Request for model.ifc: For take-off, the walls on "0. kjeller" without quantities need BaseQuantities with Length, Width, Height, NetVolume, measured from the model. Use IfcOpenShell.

First a look at what the model holds.

```python
import ifcopenshell
import ifcopenshell.util.element
import ifcopenshell.util.unit

model = ifcopenshell.open("model.ifc")
print(model.schema)
for unit_type in ("LENGTHUNIT", "AREAUNIT", "VOLUMEUNIT"):
    print(unit_type, ifcopenshell.util.unit.calculate_unit_scale(model, unit_type))
storey = next(s for s in model.by_type("IfcBuildingStorey") if s.Name == "0. kjeller")
walls = [e for e in ifcopenshell.util.element.get_decomposition(storey) if e.is_a("IfcWall")]
for e in sorted(walls, key=lambda e: e.id()):
    print(e.id(), e.is_a(), e.Name, list(ifcopenshell.util.element.get_psets(e, qtos_only=True)), sep=" | ")
```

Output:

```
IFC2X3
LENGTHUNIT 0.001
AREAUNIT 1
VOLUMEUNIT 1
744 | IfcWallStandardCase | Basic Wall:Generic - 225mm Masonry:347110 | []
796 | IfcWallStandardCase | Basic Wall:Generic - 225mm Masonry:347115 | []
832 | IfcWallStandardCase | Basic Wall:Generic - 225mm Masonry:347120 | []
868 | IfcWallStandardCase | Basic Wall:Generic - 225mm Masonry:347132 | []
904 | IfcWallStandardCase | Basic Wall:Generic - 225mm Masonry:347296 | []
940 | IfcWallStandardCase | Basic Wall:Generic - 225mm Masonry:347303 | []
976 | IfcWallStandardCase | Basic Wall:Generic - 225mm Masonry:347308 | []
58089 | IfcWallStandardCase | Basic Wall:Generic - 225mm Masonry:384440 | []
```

```python
import ifcopenshell
import ifcopenshell.api.pset
import ifcopenshell.geom
import ifcopenshell.util.element
import ifcopenshell.util.shape
import ifcopenshell.util.unit

model = ifcopenshell.open("model.ifc")
unit_scale = ifcopenshell.util.unit.calculate_unit_scale(model)
volume_scale = ifcopenshell.util.unit.calculate_unit_scale(model, "VOLUMEUNIT")
settings = ifcopenshell.geom.settings()

storey = next(s for s in model.by_type("IfcBuildingStorey") if s.Name == "0. kjeller")
walls = [e for e in ifcopenshell.util.element.get_decomposition(storey) if e.is_a("IfcWall")]

for e in sorted(walls, key=lambda e: e.id()):
    if ifcopenshell.util.element.get_psets(e, qtos_only=True, should_inherit=False):
        continue
    # Geometry comes back in metres, in the element's own axes.
    shape = ifcopenshell.geom.create_shape(settings, e)
    values = {
        "Length": ifcopenshell.util.shape.get_x(shape.geometry) / unit_scale,
        "Width": ifcopenshell.util.shape.get_y(shape.geometry) / unit_scale,
        "Height": ifcopenshell.util.shape.get_z(shape.geometry) / unit_scale,
        "NetVolume": ifcopenshell.util.shape.get_volume(shape.geometry) / volume_scale,
    }
    qto = ifcopenshell.api.pset.add_qto(model, product=e, name="BaseQuantities")
    ifcopenshell.api.pset.edit_qto(model, qto=qto, properties=values)
    print(e.id(), {k: round(v, 3) for k, v in values.items()})

model.write("model_updated.ifc")
```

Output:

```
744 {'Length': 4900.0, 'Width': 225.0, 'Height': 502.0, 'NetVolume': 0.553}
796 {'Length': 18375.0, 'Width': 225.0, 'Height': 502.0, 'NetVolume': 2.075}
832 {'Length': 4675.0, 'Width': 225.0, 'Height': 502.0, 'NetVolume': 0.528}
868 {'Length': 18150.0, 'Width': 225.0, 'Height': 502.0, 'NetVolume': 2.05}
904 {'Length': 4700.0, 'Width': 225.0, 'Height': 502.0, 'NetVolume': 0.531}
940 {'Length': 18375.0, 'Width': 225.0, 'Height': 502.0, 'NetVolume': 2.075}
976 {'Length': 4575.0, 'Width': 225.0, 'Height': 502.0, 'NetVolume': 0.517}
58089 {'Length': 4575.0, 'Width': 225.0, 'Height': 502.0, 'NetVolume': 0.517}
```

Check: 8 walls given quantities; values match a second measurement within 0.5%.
